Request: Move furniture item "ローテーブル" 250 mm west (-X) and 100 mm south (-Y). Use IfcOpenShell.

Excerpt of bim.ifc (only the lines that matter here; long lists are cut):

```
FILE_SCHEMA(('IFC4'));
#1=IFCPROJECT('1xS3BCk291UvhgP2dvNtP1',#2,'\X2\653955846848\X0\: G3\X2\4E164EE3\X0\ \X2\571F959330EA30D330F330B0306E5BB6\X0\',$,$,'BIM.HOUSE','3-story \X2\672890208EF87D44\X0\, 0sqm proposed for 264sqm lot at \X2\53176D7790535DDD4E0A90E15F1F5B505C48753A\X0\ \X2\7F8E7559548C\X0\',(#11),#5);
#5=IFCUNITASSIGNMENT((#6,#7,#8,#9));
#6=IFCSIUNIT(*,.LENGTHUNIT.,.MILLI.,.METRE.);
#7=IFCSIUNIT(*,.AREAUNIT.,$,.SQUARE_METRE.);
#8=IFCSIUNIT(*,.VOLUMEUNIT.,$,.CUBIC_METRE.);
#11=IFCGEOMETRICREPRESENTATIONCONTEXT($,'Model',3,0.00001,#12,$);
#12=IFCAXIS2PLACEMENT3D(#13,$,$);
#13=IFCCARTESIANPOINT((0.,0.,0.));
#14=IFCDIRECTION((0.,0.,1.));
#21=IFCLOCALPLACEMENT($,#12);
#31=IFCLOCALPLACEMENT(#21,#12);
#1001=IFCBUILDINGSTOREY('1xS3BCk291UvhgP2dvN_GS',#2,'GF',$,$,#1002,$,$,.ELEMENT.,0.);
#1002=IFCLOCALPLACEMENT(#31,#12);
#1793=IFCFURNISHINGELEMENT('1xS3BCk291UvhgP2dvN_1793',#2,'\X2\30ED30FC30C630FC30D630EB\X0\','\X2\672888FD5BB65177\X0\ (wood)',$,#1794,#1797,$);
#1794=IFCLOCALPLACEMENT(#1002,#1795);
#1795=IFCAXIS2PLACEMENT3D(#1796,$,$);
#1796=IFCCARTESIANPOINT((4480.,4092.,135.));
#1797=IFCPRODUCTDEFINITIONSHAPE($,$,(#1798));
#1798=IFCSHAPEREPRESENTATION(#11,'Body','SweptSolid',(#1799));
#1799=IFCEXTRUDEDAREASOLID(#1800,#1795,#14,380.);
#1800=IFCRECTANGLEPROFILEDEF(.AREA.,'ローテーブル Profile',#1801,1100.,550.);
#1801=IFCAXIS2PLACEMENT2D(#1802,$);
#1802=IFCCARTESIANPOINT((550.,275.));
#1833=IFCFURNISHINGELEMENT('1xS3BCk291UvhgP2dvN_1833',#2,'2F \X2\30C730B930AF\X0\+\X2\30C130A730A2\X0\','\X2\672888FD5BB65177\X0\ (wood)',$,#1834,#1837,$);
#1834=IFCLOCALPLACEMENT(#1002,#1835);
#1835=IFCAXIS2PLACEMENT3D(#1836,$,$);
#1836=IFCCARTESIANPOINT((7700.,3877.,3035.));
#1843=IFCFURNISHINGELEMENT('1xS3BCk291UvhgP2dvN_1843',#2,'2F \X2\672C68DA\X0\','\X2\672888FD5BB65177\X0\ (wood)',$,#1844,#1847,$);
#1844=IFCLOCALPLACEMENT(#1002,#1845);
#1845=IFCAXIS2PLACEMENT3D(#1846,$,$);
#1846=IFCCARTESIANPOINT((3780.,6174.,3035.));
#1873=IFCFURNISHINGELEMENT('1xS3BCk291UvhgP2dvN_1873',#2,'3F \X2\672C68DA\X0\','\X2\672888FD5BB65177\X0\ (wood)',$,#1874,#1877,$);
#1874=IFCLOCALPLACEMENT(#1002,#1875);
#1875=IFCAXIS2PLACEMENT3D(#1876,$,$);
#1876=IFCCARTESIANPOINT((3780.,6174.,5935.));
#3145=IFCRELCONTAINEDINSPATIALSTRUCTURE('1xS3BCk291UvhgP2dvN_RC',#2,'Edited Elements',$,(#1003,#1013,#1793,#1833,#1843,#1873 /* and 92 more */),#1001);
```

```python
import ifcopenshell
import ifcopenshell.api.geometry
import ifcopenshell.util.placement

model = ifcopenshell.open("bim.ifc")

item = model.by_guid("1xS3BCk291UvhgP2dvN_1793")
matrix = ifcopenshell.util.placement.get_local_placement(item.ObjectPlacement)
matrix[0, 3] -= 250.0
matrix[1, 3] -= 100.0
ifcopenshell.api.geometry.edit_object_placement(model, product=item, matrix=matrix, is_si=False)

print(ifcopenshell.util.placement.get_local_placement(item.ObjectPlacement).round(3) + 0.0)

model.write("bim_v2.ifc")
```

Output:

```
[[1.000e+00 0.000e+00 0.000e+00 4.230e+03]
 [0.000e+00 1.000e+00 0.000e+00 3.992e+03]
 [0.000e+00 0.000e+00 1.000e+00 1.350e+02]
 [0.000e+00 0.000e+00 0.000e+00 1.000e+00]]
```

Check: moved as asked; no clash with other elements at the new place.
